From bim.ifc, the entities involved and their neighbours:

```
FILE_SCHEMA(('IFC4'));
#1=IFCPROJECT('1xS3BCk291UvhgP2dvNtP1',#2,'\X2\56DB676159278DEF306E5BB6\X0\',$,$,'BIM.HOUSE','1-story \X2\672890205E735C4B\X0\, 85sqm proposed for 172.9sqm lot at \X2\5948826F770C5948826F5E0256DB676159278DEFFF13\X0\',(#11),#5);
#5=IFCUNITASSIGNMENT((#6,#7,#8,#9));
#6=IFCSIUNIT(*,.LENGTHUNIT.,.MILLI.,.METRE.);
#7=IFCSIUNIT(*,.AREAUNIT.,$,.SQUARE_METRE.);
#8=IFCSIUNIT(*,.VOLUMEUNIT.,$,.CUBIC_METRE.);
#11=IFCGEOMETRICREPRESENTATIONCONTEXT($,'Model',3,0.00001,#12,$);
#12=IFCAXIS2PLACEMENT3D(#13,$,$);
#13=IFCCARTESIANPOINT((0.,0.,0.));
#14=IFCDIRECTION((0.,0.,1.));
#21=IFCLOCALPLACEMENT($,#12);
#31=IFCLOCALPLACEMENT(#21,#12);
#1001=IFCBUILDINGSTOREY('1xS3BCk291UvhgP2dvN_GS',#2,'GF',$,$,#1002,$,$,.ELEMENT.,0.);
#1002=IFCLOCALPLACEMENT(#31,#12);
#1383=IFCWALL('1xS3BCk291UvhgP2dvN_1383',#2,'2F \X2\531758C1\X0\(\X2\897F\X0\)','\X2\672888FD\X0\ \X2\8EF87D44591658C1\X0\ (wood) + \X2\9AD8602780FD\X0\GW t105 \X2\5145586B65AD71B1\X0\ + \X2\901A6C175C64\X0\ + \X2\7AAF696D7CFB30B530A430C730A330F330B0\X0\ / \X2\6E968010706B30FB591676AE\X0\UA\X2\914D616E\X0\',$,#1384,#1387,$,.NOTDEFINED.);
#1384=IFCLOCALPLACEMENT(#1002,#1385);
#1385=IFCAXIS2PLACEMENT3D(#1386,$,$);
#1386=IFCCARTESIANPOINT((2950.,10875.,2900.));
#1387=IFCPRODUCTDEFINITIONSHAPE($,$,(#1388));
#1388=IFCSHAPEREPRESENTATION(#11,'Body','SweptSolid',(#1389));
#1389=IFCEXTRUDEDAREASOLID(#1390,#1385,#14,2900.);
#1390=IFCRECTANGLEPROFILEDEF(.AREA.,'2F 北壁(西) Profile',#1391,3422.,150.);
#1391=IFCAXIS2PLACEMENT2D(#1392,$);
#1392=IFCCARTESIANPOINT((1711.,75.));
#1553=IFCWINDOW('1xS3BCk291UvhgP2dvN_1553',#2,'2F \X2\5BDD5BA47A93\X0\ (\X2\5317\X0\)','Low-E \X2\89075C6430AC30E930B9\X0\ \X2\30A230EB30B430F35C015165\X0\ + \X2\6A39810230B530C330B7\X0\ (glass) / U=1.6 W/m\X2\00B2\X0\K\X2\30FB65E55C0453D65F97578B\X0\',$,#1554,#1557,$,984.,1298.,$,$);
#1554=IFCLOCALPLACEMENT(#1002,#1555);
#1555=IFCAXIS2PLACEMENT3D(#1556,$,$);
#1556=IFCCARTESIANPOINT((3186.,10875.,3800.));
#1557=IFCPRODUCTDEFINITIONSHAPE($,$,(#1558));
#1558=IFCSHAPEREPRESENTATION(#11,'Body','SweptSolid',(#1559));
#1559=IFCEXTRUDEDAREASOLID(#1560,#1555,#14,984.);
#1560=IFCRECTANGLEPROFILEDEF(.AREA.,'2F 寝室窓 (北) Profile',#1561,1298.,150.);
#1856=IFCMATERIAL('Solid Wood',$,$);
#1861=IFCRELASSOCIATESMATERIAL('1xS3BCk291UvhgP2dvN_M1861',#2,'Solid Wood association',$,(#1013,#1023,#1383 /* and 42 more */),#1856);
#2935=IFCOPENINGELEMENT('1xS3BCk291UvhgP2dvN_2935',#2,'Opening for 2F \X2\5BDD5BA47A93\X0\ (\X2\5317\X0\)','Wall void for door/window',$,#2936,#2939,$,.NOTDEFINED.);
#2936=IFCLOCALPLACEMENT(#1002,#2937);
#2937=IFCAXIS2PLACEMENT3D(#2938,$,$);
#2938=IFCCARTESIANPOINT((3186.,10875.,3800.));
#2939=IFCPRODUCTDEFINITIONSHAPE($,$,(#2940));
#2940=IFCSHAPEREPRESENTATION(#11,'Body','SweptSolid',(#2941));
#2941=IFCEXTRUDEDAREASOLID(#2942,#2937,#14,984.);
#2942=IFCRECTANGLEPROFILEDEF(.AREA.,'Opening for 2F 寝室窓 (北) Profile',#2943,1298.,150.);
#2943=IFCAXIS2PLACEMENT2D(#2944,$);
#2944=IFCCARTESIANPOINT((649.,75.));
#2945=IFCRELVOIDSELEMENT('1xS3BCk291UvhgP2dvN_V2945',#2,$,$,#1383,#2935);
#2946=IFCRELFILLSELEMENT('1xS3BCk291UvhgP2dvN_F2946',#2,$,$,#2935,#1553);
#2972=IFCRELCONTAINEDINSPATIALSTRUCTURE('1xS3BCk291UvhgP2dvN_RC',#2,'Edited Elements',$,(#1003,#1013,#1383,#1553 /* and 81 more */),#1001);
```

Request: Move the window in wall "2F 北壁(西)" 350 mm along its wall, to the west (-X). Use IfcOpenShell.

```python
import ifcopenshell
import ifcopenshell.api.geometry
import ifcopenshell.util.placement

model = ifcopenshell.open("bim.ifc")

window = model.by_id(1553)
opening = window.FillsVoids[0].RelatingOpeningElement
wall = opening.VoidsElements[0].RelatingBuildingElement

wall_matrix = ifcopenshell.util.placement.get_local_placement(wall.ObjectPlacement)
shift = wall_matrix[:3, 0] * -350.0
before = ifcopenshell.util.placement.get_local_placement(window.ObjectPlacement)[:3, 3].copy()

# The window is not placed relative to its opening, so move both.
for product in (opening, window):
    matrix = ifcopenshell.util.placement.get_local_placement(product.ObjectPlacement)
    matrix[:3, 3] += shift
    ifcopenshell.api.geometry.edit_object_placement(model, product=product, matrix=matrix, is_si=False)

after = ifcopenshell.util.placement.get_local_placement(window.ObjectPlacement)[:3, 3]
print("window moved by", (after - before).round(3) + 0.0)

model.write("bim_edited.ifc")
```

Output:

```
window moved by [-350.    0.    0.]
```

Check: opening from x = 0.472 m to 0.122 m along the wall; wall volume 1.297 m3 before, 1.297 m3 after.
